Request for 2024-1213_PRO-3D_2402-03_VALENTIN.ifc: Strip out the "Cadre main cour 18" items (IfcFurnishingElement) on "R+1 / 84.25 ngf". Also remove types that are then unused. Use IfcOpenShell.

First a look at what the model holds.

```python
import ifcopenshell
import ifcopenshell.util.element

model = ifcopenshell.open("2024-1213_PRO-3D_2402-03_VALENTIN.ifc")
print(model.schema)
storey = next(s for s in model.by_type("IfcBuildingStorey") if s.Name == "R+1 / 84.25 ngf")
furniture = [e for e in ifcopenshell.util.element.get_decomposition(storey) if e.is_a("IfcFurnishingElement")]
seen = {}
for e in furniture:
    element_type = ifcopenshell.util.element.get_type(e)
    name = element_type.Name if element_type not in (None, e) else None
    seen[name] = seen.get(name, 0) + 1
for name, count in sorted(seen.items(), key=str):
    print(count, "x", name)
```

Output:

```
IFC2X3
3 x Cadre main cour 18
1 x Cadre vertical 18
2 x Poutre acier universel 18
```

```python
import ifcopenshell
import ifcopenshell.api.root
import ifcopenshell.util.element

model = ifcopenshell.open("2024-1213_PRO-3D_2402-03_VALENTIN.ifc")

storey = next(s for s in model.by_type("IfcBuildingStorey") if s.Name == "R+1 / 84.25 ngf")
furniture = [e for e in ifcopenshell.util.element.get_decomposition(storey) if e.is_a("IfcFurnishingElement")]
targets = [e for e in furniture if (t := ifcopenshell.util.element.get_type(e)) not in (None, e) and t.Name == "Cadre main cour 18"]
types = {ifcopenshell.util.element.get_type(e) for e in targets} - {None, *targets}

for e in targets:
    ifcopenshell.api.root.remove_product(model, product=e)
print(len(targets), "removed")

unused = [t for t in types if not ifcopenshell.util.element.get_types(t)]
for t in unused:
    ifcopenshell.api.root.remove_product(model, product=t)
print(len(unused), "unused types removed")

model.write("2024-1213_PRO-3D_2402-03_VALENTIN_rev.ifc")
```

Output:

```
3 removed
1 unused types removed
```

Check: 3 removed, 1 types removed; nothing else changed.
